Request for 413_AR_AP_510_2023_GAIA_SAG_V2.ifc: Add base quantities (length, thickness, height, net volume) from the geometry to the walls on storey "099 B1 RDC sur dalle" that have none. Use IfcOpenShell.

First a look at what the model holds.

```python
import ifcopenshell
import ifcopenshell.util.element
import ifcopenshell.util.unit

model = ifcopenshell.open("413_AR_AP_510_2023_GAIA_SAG_V2.ifc")
print(model.schema)
for unit_type in ("LENGTHUNIT", "AREAUNIT", "VOLUMEUNIT"):
    print(unit_type, ifcopenshell.util.unit.calculate_unit_scale(model, unit_type))
storey = next(s for s in model.by_type("IfcBuildingStorey") if s.Name == "099 B1 RDC sur dalle")
walls = [e for e in ifcopenshell.util.element.get_decomposition(storey) if e.is_a("IfcWall")]
for e in sorted(walls, key=lambda e: e.id()):
    print(e.id(), e.is_a(), e.Name, list(ifcopenshell.util.element.get_psets(e, qtos_only=True)), sep=" | ")
```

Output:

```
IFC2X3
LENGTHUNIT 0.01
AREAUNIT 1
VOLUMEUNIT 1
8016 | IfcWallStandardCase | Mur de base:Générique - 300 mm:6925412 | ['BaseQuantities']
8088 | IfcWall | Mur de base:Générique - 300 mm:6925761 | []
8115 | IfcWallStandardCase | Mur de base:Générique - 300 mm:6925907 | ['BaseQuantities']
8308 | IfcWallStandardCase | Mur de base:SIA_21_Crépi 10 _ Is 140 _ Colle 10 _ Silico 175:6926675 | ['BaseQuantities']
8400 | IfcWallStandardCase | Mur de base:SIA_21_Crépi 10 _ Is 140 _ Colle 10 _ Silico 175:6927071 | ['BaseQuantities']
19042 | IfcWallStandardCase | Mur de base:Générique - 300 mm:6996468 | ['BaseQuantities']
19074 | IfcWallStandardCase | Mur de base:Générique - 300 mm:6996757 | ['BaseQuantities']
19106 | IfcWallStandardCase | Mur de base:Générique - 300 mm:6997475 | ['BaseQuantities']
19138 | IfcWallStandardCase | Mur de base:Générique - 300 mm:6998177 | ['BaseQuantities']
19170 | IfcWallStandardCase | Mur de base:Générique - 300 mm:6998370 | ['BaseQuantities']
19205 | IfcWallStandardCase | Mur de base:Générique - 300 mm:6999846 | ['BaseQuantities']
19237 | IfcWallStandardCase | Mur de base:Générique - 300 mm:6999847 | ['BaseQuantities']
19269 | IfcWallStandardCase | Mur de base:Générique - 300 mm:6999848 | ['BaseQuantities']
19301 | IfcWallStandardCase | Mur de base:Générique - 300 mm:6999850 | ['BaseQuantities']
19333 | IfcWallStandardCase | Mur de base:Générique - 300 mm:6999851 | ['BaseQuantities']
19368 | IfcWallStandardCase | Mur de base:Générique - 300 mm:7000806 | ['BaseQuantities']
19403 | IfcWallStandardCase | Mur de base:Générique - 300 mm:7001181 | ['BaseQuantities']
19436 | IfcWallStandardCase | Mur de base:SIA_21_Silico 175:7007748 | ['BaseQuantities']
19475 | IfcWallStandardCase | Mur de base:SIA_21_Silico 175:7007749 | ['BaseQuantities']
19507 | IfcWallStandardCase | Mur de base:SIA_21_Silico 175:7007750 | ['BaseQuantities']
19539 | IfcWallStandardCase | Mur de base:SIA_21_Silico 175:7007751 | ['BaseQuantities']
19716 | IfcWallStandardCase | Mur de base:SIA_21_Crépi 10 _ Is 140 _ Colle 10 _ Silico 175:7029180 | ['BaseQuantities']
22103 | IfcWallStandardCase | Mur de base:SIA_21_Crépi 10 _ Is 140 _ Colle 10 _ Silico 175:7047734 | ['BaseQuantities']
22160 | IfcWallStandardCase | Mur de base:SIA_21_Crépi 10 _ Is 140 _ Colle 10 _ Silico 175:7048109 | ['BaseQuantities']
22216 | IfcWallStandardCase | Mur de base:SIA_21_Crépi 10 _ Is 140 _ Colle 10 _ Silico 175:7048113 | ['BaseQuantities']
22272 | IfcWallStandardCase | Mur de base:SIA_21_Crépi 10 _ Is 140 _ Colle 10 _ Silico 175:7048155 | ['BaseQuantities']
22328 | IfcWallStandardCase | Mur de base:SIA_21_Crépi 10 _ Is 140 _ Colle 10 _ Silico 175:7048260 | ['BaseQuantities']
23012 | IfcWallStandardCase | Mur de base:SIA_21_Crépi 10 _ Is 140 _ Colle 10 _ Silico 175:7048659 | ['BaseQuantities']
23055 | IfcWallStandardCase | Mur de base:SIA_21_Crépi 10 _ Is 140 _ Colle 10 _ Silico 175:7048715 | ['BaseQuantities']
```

```python
import ifcopenshell
import ifcopenshell.api.pset
import ifcopenshell.geom
import ifcopenshell.util.element
import ifcopenshell.util.shape
import ifcopenshell.util.unit

model = ifcopenshell.open("413_AR_AP_510_2023_GAIA_SAG_V2.ifc")
unit_scale = ifcopenshell.util.unit.calculate_unit_scale(model)
volume_scale = ifcopenshell.util.unit.calculate_unit_scale(model, "VOLUMEUNIT")
settings = ifcopenshell.geom.settings()

storey = next(s for s in model.by_type("IfcBuildingStorey") if s.Name == "099 B1 RDC sur dalle")
walls = [e for e in ifcopenshell.util.element.get_decomposition(storey) if e.is_a("IfcWall")]

for e in sorted(walls, key=lambda e: e.id()):
    if ifcopenshell.util.element.get_psets(e, qtos_only=True, should_inherit=False):
        continue
    # Geometry comes back in metres, in the element's own axes.
    shape = ifcopenshell.geom.create_shape(settings, e)
    values = {
        "Length": ifcopenshell.util.shape.get_x(shape.geometry) / unit_scale,
        "Width": ifcopenshell.util.shape.get_y(shape.geometry) / unit_scale,
        "Height": ifcopenshell.util.shape.get_z(shape.geometry) / unit_scale,
        "NetVolume": ifcopenshell.util.shape.get_volume(shape.geometry) / volume_scale,
    }
    qto = ifcopenshell.api.pset.add_qto(model, product=e, name="BaseQuantities")
    ifcopenshell.api.pset.edit_qto(model, qto=qto, properties=values)
    print(e.id(), {k: round(v, 3) for k, v in values.items()})

model.write("413_AR_AP_510_2023_GAIA_SAG_V2_edited.ifc")
```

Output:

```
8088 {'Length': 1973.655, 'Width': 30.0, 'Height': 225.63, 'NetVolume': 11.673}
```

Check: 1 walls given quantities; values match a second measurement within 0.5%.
